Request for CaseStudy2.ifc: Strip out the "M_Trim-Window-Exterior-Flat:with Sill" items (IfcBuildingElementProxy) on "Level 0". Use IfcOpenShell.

First a look at what the model holds.

```python
import ifcopenshell
import ifcopenshell.util.element

model = ifcopenshell.open("CaseStudy2.ifc")
print(model.schema)
storey = next(s for s in model.by_type("IfcBuildingStorey") if s.Name == "Level 0")
proxies = [e for e in ifcopenshell.util.element.get_decomposition(storey) if e.is_a("IfcBuildingElementProxy")]
seen = {}
for e in proxies:
    element_type = ifcopenshell.util.element.get_type(e)
    name = element_type.Name if element_type not in (None, e) else None
    seen[name] = seen.get(name, 0) + 1
for name, count in sorted(seen.items(), key=str):
    print(count, "x", name)
```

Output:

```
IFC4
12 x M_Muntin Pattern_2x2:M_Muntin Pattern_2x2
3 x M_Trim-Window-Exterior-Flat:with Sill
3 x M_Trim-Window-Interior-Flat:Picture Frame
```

```python
import ifcopenshell
import ifcopenshell.api.root
import ifcopenshell.util.element

model = ifcopenshell.open("CaseStudy2.ifc")

storey = next(s for s in model.by_type("IfcBuildingStorey") if s.Name == "Level 0")
proxies = [e for e in ifcopenshell.util.element.get_decomposition(storey) if e.is_a("IfcBuildingElementProxy")]
targets = [e for e in proxies if (t := ifcopenshell.util.element.get_type(e)) not in (None, e) and t.Name == "M_Trim-Window-Exterior-Flat:with Sill"]

for e in targets:
    ifcopenshell.api.root.remove_product(model, product=e)
print(len(targets), "removed")

model.write("CaseStudy2_v2.ifc")
```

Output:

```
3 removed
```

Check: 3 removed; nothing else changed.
